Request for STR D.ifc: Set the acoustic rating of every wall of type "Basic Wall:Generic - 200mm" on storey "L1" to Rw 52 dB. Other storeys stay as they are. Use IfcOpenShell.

First a look at what the model holds.

```python
import ifcopenshell
import ifcopenshell.util.element

model = ifcopenshell.open("STR D.ifc")
print(model.schema)
storey = next(s for s in model.by_type("IfcBuildingStorey") if s.Name == "L1")
walls = [e for e in ifcopenshell.util.element.get_decomposition(storey) if e.is_a("IfcWall")]
seen = {}
for e in walls:
    element_type = ifcopenshell.util.element.get_type(e)
    key = (element_type.Name if element_type != e and element_type else None, ifcopenshell.util.element.get_pset(e, "Pset_WallCommon", "AcousticRating"))
    seen[key] = seen.get(key, 0) + 1
for (name, value), count in sorted(seen.items(), key=str):
    print(count, "x", name, "|", value)
```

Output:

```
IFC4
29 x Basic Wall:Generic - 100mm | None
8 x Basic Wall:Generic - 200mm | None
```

```python
import ifcopenshell
import ifcopenshell.api.pset
import ifcopenshell.util.element

model = ifcopenshell.open("STR D.ifc")

storey = next(s for s in model.by_type("IfcBuildingStorey") if s.Name == "L1")
walls = [e for e in ifcopenshell.util.element.get_decomposition(storey) if e.is_a("IfcWall")]

count = 0
for e in walls:
    element_type = ifcopenshell.util.element.get_type(e)
    if element_type in (None, e) or element_type.Name != "Basic Wall:Generic - 200mm":
        continue
    # add_pset returns the element's existing set when there is one.
    pset = ifcopenshell.api.pset.add_pset(model, product=e, name="Pset_WallCommon")
    ifcopenshell.api.pset.edit_pset(model, pset=pset, properties={"AcousticRating": "Rw 52 dB"})
    count += 1

print(count, "walls updated")

model.write("STR D_v2.ifc")
```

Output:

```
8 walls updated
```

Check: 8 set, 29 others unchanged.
